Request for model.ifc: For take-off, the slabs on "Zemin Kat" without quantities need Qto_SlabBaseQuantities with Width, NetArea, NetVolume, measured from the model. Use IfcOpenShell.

First a look at what the model holds.

```python
import ifcopenshell
import ifcopenshell.util.element
import ifcopenshell.util.unit

model = ifcopenshell.open("model.ifc")
print(model.schema)
for unit_type in ("LENGTHUNIT", "AREAUNIT", "VOLUMEUNIT"):
    print(unit_type, ifcopenshell.util.unit.calculate_unit_scale(model, unit_type))
storey = next(s for s in model.by_type("IfcBuildingStorey") if s.Name == "Zemin Kat")
slabs = [e for e in ifcopenshell.util.element.get_decomposition(storey) if e.is_a("IfcSlab")]
for e in sorted(slabs, key=lambda e: e.id()):
    print(e.id(), e.is_a(), e.Name, list(ifcopenshell.util.element.get_psets(e, qtos_only=True)), sep=" | ")
```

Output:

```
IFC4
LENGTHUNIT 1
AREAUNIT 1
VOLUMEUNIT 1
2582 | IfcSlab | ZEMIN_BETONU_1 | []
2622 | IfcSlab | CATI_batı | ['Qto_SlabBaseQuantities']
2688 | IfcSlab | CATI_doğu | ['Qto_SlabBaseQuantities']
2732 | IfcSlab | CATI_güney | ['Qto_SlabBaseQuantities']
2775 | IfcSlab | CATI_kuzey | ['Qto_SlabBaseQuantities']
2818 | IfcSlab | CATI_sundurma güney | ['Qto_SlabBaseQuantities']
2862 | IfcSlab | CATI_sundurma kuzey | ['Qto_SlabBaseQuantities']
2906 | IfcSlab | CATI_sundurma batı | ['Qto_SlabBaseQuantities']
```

```python
import ifcopenshell
import ifcopenshell.api.pset
import ifcopenshell.geom
import ifcopenshell.util.element
import ifcopenshell.util.shape
import ifcopenshell.util.unit

model = ifcopenshell.open("model.ifc")
unit_scale = ifcopenshell.util.unit.calculate_unit_scale(model)
area_scale = ifcopenshell.util.unit.calculate_unit_scale(model, "AREAUNIT")
volume_scale = ifcopenshell.util.unit.calculate_unit_scale(model, "VOLUMEUNIT")
settings = ifcopenshell.geom.settings()

storey = next(s for s in model.by_type("IfcBuildingStorey") if s.Name == "Zemin Kat")
slabs = [e for e in ifcopenshell.util.element.get_decomposition(storey) if e.is_a("IfcSlab")]

for e in sorted(slabs, key=lambda e: e.id()):
    if ifcopenshell.util.element.get_psets(e, qtos_only=True, should_inherit=False):
        continue
    # Geometry comes back in metres, in the element's own axes.
    shape = ifcopenshell.geom.create_shape(settings, e)
    values = {
        "Width": ifcopenshell.util.shape.get_z(shape.geometry) / unit_scale,
        "NetArea": ifcopenshell.util.shape.get_footprint_area(shape.geometry) / area_scale,
        "NetVolume": ifcopenshell.util.shape.get_volume(shape.geometry) / volume_scale,
    }
    qto = ifcopenshell.api.pset.add_qto(model, product=e, name="Qto_SlabBaseQuantities")
    ifcopenshell.api.pset.edit_qto(model, qto=qto, properties=values)
    print(e.id(), {k: round(v, 3) for k, v in values.items()})

model.write("model_rev.ifc")
```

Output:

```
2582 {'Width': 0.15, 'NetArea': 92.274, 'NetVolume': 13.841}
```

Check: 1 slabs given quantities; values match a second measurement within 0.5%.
